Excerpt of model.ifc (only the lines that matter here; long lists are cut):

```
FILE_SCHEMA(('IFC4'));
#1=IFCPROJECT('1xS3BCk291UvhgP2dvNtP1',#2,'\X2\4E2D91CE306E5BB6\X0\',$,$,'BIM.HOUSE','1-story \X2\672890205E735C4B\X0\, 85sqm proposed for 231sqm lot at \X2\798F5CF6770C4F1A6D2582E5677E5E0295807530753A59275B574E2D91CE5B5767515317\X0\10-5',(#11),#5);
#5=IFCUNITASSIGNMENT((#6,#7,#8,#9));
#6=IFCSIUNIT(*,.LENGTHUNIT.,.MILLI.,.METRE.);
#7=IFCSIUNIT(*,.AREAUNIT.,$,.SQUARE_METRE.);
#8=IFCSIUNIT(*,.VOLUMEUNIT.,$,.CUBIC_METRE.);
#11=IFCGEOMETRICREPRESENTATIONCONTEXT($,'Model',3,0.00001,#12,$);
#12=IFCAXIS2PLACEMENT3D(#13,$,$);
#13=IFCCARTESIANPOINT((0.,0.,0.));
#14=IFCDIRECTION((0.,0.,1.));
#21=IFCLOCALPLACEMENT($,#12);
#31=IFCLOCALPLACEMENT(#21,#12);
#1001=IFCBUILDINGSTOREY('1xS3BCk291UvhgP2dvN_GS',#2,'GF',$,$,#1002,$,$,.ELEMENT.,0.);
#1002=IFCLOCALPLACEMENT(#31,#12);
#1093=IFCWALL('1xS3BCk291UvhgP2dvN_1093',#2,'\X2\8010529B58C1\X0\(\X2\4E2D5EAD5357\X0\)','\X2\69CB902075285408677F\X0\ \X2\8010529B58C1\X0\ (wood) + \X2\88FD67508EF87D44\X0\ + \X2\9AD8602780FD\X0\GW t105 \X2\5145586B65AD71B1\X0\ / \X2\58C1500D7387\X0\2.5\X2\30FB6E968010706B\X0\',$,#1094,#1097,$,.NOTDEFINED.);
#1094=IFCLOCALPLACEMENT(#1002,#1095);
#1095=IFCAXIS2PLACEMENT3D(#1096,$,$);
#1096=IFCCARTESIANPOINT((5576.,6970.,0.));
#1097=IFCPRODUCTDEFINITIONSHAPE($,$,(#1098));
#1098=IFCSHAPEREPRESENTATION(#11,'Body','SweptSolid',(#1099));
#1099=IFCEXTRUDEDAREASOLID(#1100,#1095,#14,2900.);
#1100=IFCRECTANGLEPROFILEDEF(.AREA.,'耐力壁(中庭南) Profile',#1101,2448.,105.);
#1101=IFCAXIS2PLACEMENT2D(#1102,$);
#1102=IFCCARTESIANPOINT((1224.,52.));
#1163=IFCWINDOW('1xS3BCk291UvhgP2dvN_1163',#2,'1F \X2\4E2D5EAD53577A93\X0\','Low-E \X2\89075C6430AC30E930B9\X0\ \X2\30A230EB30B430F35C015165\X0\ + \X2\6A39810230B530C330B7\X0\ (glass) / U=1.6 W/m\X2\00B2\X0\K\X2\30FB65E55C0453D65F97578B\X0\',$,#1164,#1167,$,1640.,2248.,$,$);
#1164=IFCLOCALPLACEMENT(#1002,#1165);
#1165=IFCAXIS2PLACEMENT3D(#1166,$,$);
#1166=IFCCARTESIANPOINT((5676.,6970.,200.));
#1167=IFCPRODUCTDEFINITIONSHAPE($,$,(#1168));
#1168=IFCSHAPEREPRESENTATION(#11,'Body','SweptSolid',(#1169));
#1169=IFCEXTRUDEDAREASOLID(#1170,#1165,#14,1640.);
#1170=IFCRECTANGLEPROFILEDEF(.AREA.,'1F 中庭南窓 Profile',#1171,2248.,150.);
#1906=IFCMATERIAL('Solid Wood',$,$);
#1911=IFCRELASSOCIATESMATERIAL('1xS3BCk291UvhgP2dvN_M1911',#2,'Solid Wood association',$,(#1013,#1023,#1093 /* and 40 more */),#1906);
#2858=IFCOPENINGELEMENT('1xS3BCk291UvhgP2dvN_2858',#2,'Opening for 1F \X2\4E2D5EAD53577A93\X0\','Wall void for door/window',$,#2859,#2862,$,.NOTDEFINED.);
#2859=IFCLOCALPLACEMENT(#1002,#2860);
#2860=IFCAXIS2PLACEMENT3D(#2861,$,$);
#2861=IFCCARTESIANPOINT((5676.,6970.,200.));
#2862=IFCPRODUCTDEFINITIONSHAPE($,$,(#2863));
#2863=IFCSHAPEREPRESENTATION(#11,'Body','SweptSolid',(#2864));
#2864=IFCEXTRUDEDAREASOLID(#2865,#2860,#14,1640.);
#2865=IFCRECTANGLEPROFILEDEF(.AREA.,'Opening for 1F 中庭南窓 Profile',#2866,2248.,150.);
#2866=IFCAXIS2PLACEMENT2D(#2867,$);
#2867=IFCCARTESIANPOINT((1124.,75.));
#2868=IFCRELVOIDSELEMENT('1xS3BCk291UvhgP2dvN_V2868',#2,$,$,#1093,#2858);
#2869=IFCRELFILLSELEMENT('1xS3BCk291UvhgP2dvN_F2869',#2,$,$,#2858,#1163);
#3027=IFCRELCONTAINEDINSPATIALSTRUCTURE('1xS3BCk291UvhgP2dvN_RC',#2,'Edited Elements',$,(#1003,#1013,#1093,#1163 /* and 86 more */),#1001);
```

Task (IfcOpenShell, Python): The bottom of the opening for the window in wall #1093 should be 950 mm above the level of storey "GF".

```python
import numpy as np
import ifcopenshell
import ifcopenshell.api.geometry
import ifcopenshell.geom
import ifcopenshell.util.element
import ifcopenshell.util.placement
import ifcopenshell.util.shape
import ifcopenshell.util.unit

model = ifcopenshell.open("model.ifc")
unit_scale = ifcopenshell.util.unit.calculate_unit_scale(model)

window = model.by_guid("1xS3BCk291UvhgP2dvN_1163")
opening = window.FillsVoids[0].RelatingOpeningElement
storey = ifcopenshell.util.element.get_container(window, ifc_class="IfcBuildingStorey")
level = ifcopenshell.util.placement.get_local_placement(storey.ObjectPlacement)[2, 3]

# The opening's origin need not be at the sill, so measure its lowest point.
shape = ifcopenshell.geom.create_shape(ifcopenshell.geom.settings(), opening)
bottom = ifcopenshell.util.shape.get_shape_bottom_elevation(shape, shape.geometry) / unit_scale
dz = level + 950.0 - bottom

shift = np.array([0.0, 0.0, dz])
# The window is not placed relative to its opening, so move both.
for product in (opening, window):
    matrix = ifcopenshell.util.placement.get_local_placement(product.ObjectPlacement)
    matrix[:3, 3] += shift
    ifcopenshell.api.geometry.edit_object_placement(model, product=product, matrix=matrix, is_si=False)

print(f"moved by {dz * unit_scale:+.3f} m")

model.write("model_v2.ifc")
```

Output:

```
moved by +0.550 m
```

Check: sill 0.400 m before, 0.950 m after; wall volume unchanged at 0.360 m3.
